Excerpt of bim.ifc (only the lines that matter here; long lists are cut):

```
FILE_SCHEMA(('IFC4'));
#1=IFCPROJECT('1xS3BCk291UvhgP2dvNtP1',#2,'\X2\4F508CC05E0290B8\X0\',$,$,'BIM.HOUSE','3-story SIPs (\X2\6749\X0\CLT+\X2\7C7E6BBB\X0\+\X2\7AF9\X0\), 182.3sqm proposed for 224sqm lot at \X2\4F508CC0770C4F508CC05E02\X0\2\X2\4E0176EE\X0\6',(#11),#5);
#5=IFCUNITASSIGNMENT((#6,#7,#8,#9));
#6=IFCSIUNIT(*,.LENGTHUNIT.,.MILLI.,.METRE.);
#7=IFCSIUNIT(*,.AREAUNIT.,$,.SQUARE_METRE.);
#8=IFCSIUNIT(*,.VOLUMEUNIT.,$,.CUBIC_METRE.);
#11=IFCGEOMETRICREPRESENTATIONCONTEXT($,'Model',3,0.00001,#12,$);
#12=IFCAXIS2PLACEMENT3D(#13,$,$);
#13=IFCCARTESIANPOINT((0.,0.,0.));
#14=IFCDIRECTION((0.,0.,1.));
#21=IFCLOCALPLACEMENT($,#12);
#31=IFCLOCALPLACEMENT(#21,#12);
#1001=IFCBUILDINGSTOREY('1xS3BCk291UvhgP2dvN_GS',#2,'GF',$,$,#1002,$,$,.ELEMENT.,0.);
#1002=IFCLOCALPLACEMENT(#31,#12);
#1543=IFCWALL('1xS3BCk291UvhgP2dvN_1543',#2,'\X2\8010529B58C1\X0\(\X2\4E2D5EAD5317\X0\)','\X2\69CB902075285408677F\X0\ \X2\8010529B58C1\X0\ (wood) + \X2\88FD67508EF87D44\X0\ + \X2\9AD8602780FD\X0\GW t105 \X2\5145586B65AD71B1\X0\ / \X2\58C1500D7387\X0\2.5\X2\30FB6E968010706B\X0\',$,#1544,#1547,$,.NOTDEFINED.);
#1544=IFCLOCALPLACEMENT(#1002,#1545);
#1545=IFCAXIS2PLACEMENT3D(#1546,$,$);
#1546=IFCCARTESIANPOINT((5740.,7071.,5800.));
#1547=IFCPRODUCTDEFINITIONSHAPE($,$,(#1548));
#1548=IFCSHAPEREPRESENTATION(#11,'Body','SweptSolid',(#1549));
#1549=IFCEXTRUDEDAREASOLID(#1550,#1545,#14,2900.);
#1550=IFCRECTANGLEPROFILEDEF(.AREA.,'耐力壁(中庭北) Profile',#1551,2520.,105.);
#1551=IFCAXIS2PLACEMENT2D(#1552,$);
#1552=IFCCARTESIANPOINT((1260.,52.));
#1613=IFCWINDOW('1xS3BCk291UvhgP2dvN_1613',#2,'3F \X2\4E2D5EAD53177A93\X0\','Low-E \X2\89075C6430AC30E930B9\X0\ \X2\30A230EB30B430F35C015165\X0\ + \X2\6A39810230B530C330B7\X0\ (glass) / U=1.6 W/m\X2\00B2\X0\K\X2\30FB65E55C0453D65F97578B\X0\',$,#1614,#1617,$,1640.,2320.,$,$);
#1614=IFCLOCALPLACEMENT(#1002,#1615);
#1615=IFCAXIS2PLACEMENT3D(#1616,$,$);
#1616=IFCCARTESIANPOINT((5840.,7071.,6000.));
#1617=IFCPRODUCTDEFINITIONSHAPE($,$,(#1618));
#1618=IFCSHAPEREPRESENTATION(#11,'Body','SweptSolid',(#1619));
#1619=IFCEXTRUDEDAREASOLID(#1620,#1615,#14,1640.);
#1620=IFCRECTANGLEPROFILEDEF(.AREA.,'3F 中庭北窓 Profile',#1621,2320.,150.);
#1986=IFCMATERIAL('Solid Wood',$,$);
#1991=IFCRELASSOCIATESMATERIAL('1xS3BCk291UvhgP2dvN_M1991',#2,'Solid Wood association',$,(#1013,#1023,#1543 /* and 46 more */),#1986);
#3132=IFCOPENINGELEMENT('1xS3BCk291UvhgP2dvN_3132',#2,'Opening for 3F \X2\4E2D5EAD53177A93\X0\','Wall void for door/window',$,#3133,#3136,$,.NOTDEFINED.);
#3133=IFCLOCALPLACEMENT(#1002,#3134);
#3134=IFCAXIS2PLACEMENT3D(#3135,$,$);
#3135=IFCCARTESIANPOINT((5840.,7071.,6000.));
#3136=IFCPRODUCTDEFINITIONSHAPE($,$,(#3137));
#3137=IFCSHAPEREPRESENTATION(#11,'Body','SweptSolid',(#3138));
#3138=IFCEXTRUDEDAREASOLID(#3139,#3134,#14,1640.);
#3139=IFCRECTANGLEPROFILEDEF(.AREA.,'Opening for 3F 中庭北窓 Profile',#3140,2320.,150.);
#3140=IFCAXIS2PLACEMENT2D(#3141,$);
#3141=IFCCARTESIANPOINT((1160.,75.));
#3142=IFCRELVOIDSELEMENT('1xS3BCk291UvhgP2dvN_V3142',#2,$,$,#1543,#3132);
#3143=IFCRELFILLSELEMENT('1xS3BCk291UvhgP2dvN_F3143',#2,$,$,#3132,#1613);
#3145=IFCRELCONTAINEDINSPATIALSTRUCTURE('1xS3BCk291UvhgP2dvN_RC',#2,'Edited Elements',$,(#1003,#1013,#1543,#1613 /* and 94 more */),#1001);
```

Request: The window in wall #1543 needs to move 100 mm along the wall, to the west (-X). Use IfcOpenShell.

```python
import ifcopenshell
import ifcopenshell.api.geometry
import ifcopenshell.util.placement
import ifcopenshell.util.unit

model = ifcopenshell.open("bim.ifc")
unit_scale = ifcopenshell.util.unit.calculate_unit_scale(model)

window = model.by_guid("1xS3BCk291UvhgP2dvN_1613")
opening = window.FillsVoids[0].RelatingOpeningElement
wall = opening.VoidsElements[0].RelatingBuildingElement

wall_matrix = ifcopenshell.util.placement.get_local_placement(wall.ObjectPlacement)
shift = wall_matrix[:3, 0] * -0.1 / unit_scale
before = ifcopenshell.util.placement.get_local_placement(window.ObjectPlacement)[:3, 3].copy()

# The window is not placed relative to its opening, so move both.
for product in (opening, window):
    matrix = ifcopenshell.util.placement.get_local_placement(product.ObjectPlacement)
    matrix[:3, 3] += shift
    ifcopenshell.api.geometry.edit_object_placement(model, product=product, matrix=matrix, is_si=False)

after = ifcopenshell.util.placement.get_local_placement(window.ObjectPlacement)[:3, 3]
print("window moved by", (after - before).round(3) + 0.0)

model.write("bim_v2.ifc")
```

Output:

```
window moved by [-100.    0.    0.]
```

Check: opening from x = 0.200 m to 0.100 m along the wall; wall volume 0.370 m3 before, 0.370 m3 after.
